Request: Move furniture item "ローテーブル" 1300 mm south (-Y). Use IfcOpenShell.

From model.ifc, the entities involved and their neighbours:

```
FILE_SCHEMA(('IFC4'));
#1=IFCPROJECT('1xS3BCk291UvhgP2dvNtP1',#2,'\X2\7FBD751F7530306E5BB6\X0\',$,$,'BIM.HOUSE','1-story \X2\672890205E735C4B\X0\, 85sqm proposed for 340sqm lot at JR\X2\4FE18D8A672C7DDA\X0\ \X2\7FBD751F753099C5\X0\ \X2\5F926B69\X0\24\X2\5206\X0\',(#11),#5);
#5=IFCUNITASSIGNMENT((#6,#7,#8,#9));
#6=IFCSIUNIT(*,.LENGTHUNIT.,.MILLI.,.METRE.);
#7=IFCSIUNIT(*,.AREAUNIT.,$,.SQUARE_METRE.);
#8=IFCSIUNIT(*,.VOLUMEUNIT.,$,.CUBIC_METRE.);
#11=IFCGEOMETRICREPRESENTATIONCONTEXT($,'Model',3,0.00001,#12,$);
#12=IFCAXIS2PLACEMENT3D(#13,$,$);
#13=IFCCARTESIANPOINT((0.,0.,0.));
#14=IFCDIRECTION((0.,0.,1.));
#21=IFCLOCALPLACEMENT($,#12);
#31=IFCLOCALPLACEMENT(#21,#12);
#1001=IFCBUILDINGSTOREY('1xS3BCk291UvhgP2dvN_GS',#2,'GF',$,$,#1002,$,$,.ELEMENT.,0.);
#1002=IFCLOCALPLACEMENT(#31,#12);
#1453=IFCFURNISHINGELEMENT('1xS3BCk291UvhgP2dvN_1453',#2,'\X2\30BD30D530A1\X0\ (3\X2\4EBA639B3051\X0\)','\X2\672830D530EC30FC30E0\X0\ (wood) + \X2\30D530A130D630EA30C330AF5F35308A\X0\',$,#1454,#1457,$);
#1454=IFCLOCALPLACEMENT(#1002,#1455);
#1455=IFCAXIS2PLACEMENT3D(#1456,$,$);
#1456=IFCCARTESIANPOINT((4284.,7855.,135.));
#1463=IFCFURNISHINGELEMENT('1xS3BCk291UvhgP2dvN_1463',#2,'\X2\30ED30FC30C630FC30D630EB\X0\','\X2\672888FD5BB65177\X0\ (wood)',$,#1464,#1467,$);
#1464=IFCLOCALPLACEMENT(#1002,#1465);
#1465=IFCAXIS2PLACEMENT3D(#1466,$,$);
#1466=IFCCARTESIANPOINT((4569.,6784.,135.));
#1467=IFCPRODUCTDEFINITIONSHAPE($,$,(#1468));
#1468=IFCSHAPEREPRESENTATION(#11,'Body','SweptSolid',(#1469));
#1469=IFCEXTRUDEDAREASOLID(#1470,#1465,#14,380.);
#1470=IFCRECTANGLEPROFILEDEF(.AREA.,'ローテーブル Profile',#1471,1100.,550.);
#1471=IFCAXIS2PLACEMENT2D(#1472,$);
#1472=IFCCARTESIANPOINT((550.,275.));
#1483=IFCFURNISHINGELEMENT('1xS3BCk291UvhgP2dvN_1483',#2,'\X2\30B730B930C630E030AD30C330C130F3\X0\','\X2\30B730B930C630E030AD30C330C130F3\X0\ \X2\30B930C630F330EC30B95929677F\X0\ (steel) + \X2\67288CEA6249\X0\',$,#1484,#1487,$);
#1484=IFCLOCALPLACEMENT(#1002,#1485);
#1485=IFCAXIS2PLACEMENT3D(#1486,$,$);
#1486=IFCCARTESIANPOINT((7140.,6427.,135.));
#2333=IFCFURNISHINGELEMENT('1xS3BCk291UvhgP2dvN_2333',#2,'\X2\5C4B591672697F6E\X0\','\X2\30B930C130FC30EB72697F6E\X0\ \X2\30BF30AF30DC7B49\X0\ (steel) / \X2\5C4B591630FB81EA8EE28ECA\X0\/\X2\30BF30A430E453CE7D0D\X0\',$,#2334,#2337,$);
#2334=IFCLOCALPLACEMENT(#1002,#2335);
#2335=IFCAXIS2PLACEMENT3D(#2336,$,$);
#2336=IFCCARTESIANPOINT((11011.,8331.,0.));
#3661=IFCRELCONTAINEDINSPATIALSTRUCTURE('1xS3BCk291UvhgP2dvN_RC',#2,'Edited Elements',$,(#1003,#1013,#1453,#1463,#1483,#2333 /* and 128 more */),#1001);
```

```python
import ifcopenshell
import ifcopenshell.api.geometry
import ifcopenshell.util.placement
import ifcopenshell.util.unit

model = ifcopenshell.open("model.ifc")
unit_scale = ifcopenshell.util.unit.calculate_unit_scale(model)

item = model.by_guid("1xS3BCk291UvhgP2dvN_1463")
matrix = ifcopenshell.util.placement.get_local_placement(item.ObjectPlacement)
matrix[1, 3] -= 1.3 / unit_scale
ifcopenshell.api.geometry.edit_object_placement(model, product=item, matrix=matrix, is_si=False)

print(ifcopenshell.util.placement.get_local_placement(item.ObjectPlacement).round(3) + 0.0)

model.write("model_edited.ifc")
```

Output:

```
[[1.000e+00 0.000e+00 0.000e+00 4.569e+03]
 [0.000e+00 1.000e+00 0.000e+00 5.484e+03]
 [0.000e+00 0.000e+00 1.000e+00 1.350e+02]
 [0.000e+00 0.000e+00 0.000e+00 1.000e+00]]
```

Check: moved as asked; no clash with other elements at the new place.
